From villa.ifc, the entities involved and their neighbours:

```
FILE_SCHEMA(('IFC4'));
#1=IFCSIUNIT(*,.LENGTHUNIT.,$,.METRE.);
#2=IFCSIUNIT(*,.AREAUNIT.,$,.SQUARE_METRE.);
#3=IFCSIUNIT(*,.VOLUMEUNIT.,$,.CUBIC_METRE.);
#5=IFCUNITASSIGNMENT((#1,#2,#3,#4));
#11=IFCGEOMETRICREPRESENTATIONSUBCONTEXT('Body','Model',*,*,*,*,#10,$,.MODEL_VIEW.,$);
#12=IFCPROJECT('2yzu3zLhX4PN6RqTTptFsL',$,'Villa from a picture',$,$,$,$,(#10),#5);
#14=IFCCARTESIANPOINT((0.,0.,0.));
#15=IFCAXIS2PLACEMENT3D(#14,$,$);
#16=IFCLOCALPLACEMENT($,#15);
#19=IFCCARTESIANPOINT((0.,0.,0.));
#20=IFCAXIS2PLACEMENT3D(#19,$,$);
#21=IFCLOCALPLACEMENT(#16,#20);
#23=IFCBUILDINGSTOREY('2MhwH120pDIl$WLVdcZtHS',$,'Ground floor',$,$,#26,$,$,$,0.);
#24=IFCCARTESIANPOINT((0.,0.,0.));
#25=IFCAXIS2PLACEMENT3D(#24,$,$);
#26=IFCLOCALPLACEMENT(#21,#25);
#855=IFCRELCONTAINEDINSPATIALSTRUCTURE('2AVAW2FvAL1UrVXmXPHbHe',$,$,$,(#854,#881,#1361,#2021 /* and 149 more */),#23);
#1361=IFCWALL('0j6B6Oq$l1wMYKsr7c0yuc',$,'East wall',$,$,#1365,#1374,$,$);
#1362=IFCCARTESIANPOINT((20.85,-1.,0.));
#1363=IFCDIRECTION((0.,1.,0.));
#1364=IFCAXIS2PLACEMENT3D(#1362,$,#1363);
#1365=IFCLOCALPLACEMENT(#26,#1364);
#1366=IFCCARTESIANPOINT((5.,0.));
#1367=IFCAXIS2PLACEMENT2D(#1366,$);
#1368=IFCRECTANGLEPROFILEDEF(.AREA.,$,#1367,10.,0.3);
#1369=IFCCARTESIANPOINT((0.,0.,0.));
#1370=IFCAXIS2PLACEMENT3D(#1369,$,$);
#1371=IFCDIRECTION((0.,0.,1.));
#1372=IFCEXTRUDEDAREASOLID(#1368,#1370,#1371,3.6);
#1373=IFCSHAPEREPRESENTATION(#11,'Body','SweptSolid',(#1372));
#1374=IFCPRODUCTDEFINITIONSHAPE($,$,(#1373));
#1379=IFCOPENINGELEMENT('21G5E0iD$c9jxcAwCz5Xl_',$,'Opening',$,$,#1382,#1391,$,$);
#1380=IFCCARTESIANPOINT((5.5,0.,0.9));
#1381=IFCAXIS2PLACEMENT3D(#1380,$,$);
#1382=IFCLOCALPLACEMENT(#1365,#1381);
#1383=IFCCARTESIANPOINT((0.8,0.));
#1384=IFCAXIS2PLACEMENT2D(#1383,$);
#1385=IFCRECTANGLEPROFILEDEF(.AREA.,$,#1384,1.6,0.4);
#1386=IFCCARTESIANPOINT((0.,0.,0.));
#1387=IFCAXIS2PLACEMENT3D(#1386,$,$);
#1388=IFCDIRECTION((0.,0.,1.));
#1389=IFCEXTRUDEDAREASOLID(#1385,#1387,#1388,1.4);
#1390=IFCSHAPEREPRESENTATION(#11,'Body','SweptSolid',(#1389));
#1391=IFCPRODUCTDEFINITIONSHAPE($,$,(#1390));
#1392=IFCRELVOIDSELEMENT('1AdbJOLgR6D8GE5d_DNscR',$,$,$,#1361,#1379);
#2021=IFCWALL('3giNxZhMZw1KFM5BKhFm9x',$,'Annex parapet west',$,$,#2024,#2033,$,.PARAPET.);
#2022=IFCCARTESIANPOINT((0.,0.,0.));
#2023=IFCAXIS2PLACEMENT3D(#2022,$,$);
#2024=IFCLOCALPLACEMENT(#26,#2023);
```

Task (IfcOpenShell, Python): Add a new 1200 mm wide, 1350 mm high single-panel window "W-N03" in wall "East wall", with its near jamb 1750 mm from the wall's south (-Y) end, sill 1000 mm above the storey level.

```python
import numpy as np
import ifcopenshell
import ifcopenshell.api.feature
import ifcopenshell.api.geometry
import ifcopenshell.api.root
import ifcopenshell.api.spatial
import ifcopenshell.geom
import ifcopenshell.util.element
import ifcopenshell.util.placement
import ifcopenshell.util.representation
import ifcopenshell.util.shape
import ifcopenshell.util.unit

model = ifcopenshell.open("villa.ifc")
unit_scale = ifcopenshell.util.unit.calculate_unit_scale(model)
settings = ifcopenshell.geom.settings()


def volume(element):
    """Net volume in cubic metres, openings subtracted."""
    shape = ifcopenshell.geom.create_shape(settings, element)
    return ifcopenshell.util.shape.get_volume(shape.geometry)


wall = model.by_id(1361)
storey = ifcopenshell.util.element.get_container(wall, ifc_class="IfcBuildingStorey")
context = ifcopenshell.util.representation.get_context(model, "Model", "Body", "MODEL_VIEW")
before = volume(wall)

width, height, from_end, sill = 1.2, 1.35, 1.75, 1  # metres

# The wall runs along its own X axis, and the end named is its -X end.
wall_shape = ifcopenshell.geom.create_shape(settings, wall)
x, y, z = ifcopenshell.util.shape.get_vertices(wall_shape.geometry).T
start = x.min() + from_end
face, thickness = float(y.min()), float(y.max() - y.min())
wall_matrix = ifcopenshell.util.placement.get_local_placement(wall.ObjectPlacement)
level = ifcopenshell.util.placement.get_local_placement(storey.ObjectPlacement)[2, 3]


def in_wall(x, y):
    """Placement at x, y metres in the wall's axes, at sill height."""
    matrix = wall_matrix.copy()
    matrix[:, 3] = wall_matrix @ np.array([x / unit_scale, y / unit_scale, 0.0, 1.0])
    matrix[2, 3] = level + sill / unit_scale
    return matrix


# Opening: a box that overshoots both wall faces by 50 mm.
opening = ifcopenshell.api.root.create_entity(model, ifc_class="IfcOpeningElement", predefined_type="OPENING")
box = ifcopenshell.api.geometry.add_wall_representation(
    model, context=context, length=width, height=height, thickness=thickness + 0.1
)
ifcopenshell.api.geometry.assign_representation(model, product=opening, representation=box)
ifcopenshell.api.geometry.edit_object_placement(model, product=opening, matrix=in_wall(start, face - 0.05), is_si=False)
ifcopenshell.api.feature.add_feature(model, feature=opening, element=wall)

window = ifcopenshell.api.root.create_entity(model, ifc_class="IfcWindow", name="W-N03", predefined_type="WINDOW")
window.OverallWidth, window.OverallHeight = width / unit_scale, height / unit_scale
window.PartitioningType = "SINGLE_PANEL"
body = ifcopenshell.api.geometry.add_window_representation(
    model,
    context=context,
    overall_width=window.OverallWidth,
    overall_height=window.OverallHeight,
    partition_type="SINGLE_PANEL",
)
ifcopenshell.api.geometry.assign_representation(model, product=window, representation=body)
ifcopenshell.api.spatial.assign_container(model, products=[window], relating_structure=storey)
ifcopenshell.api.feature.add_filling(model, opening=opening, element=window)

# Centre the window in the wall's thickness.
ifcopenshell.api.geometry.edit_object_placement(model, product=window, matrix=in_wall(start, face), is_si=False)
window_shape = ifcopenshell.geom.create_shape(settings, window)
depth = ifcopenshell.util.shape.get_vertices(window_shape.geometry)[:, 1]
offset = face + thickness / 2 - (depth.min() + depth.max()) / 2
ifcopenshell.api.geometry.edit_object_placement(model, product=window, matrix=in_wall(start, offset), is_si=False)

after = volume(wall)

print(f"wall volume {before:.3f} -> {after:.3f} m3")

model.write("villa_updated.ifc")
```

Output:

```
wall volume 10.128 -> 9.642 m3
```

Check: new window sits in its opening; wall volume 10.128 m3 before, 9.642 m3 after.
